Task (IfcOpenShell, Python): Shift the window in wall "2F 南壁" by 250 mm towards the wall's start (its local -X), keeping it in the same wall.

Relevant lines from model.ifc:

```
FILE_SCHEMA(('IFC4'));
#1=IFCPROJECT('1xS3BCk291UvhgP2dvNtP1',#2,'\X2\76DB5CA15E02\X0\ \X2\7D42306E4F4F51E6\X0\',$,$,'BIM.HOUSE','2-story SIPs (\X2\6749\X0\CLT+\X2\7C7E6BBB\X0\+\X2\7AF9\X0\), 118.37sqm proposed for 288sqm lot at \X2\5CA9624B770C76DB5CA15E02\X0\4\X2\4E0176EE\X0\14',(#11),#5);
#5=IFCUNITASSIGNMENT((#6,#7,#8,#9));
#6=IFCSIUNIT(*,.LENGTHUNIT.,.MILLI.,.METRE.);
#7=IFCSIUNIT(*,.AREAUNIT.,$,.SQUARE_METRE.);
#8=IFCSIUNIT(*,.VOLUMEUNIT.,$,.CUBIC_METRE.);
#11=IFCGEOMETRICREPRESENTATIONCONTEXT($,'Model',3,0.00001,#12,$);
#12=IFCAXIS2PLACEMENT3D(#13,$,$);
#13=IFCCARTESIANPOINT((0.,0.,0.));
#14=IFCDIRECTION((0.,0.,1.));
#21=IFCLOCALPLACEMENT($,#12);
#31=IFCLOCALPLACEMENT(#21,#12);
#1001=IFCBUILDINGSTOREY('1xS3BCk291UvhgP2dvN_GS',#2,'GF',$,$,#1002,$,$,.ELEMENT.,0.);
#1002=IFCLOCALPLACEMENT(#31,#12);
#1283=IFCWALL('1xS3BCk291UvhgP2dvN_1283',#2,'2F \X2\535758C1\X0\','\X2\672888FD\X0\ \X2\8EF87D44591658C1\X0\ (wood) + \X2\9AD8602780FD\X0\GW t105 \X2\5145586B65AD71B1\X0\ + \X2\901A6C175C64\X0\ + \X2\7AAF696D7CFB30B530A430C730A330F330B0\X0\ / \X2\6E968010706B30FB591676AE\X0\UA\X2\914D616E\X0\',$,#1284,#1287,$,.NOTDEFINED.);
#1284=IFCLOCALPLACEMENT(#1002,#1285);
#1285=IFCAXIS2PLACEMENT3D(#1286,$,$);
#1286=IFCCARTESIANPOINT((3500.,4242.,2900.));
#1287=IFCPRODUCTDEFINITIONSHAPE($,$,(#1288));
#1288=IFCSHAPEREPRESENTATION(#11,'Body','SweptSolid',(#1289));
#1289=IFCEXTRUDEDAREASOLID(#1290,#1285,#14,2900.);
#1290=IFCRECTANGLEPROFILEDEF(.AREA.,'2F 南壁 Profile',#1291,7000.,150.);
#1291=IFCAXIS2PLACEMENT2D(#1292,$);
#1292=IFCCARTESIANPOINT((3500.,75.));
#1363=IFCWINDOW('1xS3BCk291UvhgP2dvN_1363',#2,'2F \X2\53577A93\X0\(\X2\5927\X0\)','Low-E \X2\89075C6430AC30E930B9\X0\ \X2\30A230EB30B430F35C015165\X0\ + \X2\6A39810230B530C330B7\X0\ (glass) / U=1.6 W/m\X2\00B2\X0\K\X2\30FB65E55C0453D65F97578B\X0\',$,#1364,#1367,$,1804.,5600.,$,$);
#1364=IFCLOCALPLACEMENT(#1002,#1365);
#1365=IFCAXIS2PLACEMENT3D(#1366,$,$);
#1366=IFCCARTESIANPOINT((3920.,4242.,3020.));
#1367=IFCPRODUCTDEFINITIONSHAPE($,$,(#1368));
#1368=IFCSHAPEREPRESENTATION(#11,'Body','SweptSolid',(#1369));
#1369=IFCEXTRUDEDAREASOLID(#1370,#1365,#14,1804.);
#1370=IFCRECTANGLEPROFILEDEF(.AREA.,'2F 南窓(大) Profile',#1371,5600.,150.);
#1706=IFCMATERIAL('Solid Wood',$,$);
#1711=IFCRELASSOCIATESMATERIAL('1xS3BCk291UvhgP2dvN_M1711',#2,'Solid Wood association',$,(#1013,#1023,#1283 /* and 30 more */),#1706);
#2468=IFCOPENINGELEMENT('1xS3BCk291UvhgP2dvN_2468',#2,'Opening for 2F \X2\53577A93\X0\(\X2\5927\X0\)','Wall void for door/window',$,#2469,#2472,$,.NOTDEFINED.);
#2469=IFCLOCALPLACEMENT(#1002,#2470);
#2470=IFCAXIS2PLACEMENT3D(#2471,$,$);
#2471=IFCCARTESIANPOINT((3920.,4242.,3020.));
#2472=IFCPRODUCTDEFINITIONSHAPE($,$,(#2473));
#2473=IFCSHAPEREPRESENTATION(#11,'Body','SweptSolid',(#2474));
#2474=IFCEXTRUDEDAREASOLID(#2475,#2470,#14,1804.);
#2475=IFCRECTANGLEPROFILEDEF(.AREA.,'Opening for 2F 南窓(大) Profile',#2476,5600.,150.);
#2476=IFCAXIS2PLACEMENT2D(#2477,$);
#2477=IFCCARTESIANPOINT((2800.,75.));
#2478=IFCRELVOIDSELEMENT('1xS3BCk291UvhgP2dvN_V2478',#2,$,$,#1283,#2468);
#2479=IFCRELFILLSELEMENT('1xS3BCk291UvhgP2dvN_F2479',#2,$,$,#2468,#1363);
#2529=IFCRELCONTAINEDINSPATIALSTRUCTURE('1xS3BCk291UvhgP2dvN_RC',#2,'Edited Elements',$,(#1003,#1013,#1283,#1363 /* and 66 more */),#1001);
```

```python
import ifcopenshell
import ifcopenshell.api.geometry
import ifcopenshell.util.placement

model = ifcopenshell.open("model.ifc")

window = model.by_guid("1xS3BCk291UvhgP2dvN_1363")
opening = window.FillsVoids[0].RelatingOpeningElement
wall = opening.VoidsElements[0].RelatingBuildingElement

wall_matrix = ifcopenshell.util.placement.get_local_placement(wall.ObjectPlacement)
shift = wall_matrix[:3, 0] * -250.0
before = ifcopenshell.util.placement.get_local_placement(window.ObjectPlacement)[:3, 3].copy()

# The window is not placed relative to its opening, so move both.
for product in (opening, window):
    matrix = ifcopenshell.util.placement.get_local_placement(product.ObjectPlacement)
    matrix[:3, 3] += shift
    ifcopenshell.api.geometry.edit_object_placement(model, product=product, matrix=matrix, is_si=False)

after = ifcopenshell.util.placement.get_local_placement(window.ObjectPlacement)[:3, 3]
print("window moved by", (after - before).round(3) + 0.0)

model.write("model-out.ifc")
```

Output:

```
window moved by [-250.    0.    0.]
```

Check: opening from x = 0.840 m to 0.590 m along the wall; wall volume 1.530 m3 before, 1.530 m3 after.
